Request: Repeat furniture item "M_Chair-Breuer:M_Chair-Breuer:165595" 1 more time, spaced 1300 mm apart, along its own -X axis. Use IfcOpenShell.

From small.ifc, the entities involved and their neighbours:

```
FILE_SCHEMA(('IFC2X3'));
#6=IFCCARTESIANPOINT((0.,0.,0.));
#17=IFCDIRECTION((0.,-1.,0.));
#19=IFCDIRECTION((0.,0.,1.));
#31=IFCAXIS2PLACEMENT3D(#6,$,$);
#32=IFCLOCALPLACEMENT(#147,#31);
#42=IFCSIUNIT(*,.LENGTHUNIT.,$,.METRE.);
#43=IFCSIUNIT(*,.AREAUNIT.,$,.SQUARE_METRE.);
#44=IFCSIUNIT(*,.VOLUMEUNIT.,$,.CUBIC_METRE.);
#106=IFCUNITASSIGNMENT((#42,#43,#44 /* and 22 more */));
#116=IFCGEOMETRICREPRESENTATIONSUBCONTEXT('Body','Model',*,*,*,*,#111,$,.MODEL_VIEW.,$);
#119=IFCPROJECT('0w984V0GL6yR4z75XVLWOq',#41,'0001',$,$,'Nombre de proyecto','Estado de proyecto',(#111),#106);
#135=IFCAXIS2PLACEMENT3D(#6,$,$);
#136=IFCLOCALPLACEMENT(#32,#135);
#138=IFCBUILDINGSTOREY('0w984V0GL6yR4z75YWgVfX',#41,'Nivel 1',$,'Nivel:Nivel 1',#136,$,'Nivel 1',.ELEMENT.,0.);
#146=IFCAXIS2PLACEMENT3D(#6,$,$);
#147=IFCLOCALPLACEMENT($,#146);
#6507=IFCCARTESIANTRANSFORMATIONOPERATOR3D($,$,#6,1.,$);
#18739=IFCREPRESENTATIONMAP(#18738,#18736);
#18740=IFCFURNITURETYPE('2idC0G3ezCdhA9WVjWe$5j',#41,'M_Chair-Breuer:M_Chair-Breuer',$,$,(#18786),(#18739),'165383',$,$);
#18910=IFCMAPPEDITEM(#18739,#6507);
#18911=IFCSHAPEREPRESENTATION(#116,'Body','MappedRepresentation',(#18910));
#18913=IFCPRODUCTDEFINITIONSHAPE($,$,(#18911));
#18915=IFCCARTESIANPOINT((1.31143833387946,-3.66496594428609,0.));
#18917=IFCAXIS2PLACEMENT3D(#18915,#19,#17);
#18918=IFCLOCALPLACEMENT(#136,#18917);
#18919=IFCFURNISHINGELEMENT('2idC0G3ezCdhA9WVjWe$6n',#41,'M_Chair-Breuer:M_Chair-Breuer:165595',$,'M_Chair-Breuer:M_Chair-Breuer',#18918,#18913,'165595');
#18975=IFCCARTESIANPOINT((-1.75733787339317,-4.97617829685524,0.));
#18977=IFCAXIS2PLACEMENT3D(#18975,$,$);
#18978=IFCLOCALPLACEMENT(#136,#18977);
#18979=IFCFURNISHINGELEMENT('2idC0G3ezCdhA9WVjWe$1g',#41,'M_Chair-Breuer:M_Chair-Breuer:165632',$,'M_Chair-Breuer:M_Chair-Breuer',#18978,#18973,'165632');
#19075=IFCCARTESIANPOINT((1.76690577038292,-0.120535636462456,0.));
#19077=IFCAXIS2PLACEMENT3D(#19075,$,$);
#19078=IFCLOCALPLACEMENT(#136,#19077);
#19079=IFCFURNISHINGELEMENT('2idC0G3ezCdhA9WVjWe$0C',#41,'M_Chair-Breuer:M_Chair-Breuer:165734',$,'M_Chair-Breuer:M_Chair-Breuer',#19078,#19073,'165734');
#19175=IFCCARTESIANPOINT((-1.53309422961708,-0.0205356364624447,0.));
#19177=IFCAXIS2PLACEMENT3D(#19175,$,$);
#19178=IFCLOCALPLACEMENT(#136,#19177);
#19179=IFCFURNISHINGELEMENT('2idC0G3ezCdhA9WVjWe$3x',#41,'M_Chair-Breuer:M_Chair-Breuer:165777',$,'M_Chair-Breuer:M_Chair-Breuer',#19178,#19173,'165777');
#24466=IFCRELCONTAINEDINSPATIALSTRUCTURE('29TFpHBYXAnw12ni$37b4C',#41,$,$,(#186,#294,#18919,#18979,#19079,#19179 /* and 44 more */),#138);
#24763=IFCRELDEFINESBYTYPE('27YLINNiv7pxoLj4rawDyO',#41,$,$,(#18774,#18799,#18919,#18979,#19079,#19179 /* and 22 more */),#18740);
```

```python
import ifcopenshell
import ifcopenshell.api.geometry
import ifcopenshell.api.root
import ifcopenshell.util.element
import ifcopenshell.util.placement

model = ifcopenshell.open("small.ifc")


def reuse_history(source, copy):
    """copy_class also copies each property set's owner history, people and application; keep the originals."""
    for rel in copy.IsDefinedBy:
        if rel.is_a("IfcRelDefinesByProperties") and (history := rel.RelatingPropertyDefinition.OwnerHistory):
            rel.RelatingPropertyDefinition.OwnerHistory = source.OwnerHistory
            ifcopenshell.util.element.remove_deep2(model, history)


source = model.by_id(18919)
base = ifcopenshell.util.placement.get_local_placement(source.ObjectPlacement)
step = -base[:3, 0] * 1.3

for i in range(1, 2):
    copy = ifcopenshell.api.root.copy_class(model, product=source)
    copy.Representation = ifcopenshell.util.element.copy_deep(
        model, source.Representation, exclude=["IfcGeometricRepresentationContext", "IfcRepresentationMap"]
    )
    copy.Name = "M_Chair-Breuer:M_Chair-Breuer"
    copy.Tag = None
    reuse_history(source, copy)
    matrix = base.copy()
    matrix[:3, 3] += i * step
    print("added at", matrix[:3, 3].round(3) + 0.0)
    ifcopenshell.api.geometry.edit_object_placement(model, product=copy, matrix=matrix, is_si=False)

model.write("small_v2.ifc")
```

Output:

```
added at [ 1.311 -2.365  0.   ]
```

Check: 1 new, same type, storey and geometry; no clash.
